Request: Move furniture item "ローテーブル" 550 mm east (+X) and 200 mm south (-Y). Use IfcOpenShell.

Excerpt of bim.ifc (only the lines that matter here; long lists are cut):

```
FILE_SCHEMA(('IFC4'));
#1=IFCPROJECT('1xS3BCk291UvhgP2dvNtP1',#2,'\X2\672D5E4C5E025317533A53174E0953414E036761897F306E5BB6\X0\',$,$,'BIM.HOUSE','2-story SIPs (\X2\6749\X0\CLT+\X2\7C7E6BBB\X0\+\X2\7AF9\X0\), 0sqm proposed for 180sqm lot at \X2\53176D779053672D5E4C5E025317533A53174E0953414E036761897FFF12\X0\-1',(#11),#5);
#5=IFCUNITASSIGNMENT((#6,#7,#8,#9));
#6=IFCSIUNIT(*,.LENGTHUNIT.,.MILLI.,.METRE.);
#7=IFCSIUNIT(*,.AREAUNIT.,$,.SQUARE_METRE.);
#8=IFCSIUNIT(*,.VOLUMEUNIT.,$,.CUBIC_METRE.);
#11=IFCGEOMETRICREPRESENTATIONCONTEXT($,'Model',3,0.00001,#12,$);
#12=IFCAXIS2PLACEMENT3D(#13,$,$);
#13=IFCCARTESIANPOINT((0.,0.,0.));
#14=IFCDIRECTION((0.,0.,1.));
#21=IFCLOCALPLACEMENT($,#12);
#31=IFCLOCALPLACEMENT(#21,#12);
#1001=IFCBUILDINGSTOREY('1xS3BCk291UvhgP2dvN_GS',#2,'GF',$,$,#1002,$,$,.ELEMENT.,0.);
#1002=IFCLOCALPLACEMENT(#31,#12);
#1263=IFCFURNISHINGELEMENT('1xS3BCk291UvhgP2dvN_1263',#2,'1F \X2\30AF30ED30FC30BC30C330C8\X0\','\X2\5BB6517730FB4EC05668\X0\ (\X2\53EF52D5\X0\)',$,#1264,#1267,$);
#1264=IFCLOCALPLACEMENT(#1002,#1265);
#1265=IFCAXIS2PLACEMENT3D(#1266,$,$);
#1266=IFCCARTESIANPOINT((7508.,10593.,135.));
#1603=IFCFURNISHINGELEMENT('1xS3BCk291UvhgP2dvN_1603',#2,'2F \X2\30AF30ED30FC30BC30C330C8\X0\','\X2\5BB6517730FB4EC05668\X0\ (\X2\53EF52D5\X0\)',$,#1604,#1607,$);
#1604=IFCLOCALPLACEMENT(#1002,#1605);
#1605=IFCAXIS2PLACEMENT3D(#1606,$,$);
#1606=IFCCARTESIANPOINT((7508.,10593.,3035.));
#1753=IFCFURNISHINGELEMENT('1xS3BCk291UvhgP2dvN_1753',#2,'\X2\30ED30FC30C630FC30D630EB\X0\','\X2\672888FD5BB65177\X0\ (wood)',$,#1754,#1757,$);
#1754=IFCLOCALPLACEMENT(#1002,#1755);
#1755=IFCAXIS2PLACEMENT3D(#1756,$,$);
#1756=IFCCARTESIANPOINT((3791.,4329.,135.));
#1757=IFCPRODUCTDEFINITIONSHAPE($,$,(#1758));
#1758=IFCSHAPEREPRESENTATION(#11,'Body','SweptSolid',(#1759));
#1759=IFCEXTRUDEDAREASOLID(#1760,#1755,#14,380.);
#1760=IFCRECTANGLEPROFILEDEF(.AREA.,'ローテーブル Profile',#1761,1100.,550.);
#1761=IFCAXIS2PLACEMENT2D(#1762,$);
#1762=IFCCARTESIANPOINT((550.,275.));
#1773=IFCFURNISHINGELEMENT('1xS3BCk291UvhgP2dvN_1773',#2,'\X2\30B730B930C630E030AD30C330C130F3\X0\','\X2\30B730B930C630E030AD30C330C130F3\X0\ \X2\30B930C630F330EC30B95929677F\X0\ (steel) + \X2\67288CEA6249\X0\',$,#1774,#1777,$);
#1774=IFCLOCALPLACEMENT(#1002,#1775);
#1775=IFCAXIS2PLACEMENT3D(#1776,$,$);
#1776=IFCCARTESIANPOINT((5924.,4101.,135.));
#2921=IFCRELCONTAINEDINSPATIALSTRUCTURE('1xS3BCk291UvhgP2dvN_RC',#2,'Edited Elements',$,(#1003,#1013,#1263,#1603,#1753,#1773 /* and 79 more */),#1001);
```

```python
import ifcopenshell
import ifcopenshell.api.geometry
import ifcopenshell.util.placement

model = ifcopenshell.open("bim.ifc")

item = model.by_id(1753)
matrix = ifcopenshell.util.placement.get_local_placement(item.ObjectPlacement)
matrix[0, 3] += 550.0
matrix[1, 3] -= 200.0
ifcopenshell.api.geometry.edit_object_placement(model, product=item, matrix=matrix, is_si=False)

print(ifcopenshell.util.placement.get_local_placement(item.ObjectPlacement).round(3) + 0.0)

model.write("bim_edited.ifc")
```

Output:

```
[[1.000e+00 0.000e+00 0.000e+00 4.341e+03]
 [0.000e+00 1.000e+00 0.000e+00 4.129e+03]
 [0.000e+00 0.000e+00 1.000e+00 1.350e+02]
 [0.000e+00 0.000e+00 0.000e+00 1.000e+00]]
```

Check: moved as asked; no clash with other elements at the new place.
